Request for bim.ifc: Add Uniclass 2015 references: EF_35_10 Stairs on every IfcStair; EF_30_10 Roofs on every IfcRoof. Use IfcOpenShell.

First a look at what the model holds.

```python
import ifcopenshell

model = ifcopenshell.open("bim.ifc")
print(model.schema)
print("classifications:", [c.Name for c in model.by_type("IfcClassification")])
for ifc_class in ("IfcDoor", "IfcRoof", "IfcStair", "IfcWall", "IfcWindow"):
    print(ifc_class, len(model.by_type(ifc_class)))
```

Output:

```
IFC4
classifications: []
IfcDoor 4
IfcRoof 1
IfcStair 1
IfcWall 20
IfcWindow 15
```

```python
import ifcopenshell
import ifcopenshell.api.classification

model = ifcopenshell.open("bim.ifc")

system = ifcopenshell.api.classification.add_classification(model, classification="Uniclass 2015")

codes = {
    "IfcStair": ("EF_35_10", "Stairs"),
    "IfcRoof": ("EF_30_10", "Roofs"),
}
for ifc_class, (code, name) in codes.items():
    products = model.by_type(ifc_class)
    ifcopenshell.api.classification.add_reference(
        model, products=products, classification=system, identification=code, name=name
    )
    print(code, len(products))

model.write("bim_v2.ifc")
```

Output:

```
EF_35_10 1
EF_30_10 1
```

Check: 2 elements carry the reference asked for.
